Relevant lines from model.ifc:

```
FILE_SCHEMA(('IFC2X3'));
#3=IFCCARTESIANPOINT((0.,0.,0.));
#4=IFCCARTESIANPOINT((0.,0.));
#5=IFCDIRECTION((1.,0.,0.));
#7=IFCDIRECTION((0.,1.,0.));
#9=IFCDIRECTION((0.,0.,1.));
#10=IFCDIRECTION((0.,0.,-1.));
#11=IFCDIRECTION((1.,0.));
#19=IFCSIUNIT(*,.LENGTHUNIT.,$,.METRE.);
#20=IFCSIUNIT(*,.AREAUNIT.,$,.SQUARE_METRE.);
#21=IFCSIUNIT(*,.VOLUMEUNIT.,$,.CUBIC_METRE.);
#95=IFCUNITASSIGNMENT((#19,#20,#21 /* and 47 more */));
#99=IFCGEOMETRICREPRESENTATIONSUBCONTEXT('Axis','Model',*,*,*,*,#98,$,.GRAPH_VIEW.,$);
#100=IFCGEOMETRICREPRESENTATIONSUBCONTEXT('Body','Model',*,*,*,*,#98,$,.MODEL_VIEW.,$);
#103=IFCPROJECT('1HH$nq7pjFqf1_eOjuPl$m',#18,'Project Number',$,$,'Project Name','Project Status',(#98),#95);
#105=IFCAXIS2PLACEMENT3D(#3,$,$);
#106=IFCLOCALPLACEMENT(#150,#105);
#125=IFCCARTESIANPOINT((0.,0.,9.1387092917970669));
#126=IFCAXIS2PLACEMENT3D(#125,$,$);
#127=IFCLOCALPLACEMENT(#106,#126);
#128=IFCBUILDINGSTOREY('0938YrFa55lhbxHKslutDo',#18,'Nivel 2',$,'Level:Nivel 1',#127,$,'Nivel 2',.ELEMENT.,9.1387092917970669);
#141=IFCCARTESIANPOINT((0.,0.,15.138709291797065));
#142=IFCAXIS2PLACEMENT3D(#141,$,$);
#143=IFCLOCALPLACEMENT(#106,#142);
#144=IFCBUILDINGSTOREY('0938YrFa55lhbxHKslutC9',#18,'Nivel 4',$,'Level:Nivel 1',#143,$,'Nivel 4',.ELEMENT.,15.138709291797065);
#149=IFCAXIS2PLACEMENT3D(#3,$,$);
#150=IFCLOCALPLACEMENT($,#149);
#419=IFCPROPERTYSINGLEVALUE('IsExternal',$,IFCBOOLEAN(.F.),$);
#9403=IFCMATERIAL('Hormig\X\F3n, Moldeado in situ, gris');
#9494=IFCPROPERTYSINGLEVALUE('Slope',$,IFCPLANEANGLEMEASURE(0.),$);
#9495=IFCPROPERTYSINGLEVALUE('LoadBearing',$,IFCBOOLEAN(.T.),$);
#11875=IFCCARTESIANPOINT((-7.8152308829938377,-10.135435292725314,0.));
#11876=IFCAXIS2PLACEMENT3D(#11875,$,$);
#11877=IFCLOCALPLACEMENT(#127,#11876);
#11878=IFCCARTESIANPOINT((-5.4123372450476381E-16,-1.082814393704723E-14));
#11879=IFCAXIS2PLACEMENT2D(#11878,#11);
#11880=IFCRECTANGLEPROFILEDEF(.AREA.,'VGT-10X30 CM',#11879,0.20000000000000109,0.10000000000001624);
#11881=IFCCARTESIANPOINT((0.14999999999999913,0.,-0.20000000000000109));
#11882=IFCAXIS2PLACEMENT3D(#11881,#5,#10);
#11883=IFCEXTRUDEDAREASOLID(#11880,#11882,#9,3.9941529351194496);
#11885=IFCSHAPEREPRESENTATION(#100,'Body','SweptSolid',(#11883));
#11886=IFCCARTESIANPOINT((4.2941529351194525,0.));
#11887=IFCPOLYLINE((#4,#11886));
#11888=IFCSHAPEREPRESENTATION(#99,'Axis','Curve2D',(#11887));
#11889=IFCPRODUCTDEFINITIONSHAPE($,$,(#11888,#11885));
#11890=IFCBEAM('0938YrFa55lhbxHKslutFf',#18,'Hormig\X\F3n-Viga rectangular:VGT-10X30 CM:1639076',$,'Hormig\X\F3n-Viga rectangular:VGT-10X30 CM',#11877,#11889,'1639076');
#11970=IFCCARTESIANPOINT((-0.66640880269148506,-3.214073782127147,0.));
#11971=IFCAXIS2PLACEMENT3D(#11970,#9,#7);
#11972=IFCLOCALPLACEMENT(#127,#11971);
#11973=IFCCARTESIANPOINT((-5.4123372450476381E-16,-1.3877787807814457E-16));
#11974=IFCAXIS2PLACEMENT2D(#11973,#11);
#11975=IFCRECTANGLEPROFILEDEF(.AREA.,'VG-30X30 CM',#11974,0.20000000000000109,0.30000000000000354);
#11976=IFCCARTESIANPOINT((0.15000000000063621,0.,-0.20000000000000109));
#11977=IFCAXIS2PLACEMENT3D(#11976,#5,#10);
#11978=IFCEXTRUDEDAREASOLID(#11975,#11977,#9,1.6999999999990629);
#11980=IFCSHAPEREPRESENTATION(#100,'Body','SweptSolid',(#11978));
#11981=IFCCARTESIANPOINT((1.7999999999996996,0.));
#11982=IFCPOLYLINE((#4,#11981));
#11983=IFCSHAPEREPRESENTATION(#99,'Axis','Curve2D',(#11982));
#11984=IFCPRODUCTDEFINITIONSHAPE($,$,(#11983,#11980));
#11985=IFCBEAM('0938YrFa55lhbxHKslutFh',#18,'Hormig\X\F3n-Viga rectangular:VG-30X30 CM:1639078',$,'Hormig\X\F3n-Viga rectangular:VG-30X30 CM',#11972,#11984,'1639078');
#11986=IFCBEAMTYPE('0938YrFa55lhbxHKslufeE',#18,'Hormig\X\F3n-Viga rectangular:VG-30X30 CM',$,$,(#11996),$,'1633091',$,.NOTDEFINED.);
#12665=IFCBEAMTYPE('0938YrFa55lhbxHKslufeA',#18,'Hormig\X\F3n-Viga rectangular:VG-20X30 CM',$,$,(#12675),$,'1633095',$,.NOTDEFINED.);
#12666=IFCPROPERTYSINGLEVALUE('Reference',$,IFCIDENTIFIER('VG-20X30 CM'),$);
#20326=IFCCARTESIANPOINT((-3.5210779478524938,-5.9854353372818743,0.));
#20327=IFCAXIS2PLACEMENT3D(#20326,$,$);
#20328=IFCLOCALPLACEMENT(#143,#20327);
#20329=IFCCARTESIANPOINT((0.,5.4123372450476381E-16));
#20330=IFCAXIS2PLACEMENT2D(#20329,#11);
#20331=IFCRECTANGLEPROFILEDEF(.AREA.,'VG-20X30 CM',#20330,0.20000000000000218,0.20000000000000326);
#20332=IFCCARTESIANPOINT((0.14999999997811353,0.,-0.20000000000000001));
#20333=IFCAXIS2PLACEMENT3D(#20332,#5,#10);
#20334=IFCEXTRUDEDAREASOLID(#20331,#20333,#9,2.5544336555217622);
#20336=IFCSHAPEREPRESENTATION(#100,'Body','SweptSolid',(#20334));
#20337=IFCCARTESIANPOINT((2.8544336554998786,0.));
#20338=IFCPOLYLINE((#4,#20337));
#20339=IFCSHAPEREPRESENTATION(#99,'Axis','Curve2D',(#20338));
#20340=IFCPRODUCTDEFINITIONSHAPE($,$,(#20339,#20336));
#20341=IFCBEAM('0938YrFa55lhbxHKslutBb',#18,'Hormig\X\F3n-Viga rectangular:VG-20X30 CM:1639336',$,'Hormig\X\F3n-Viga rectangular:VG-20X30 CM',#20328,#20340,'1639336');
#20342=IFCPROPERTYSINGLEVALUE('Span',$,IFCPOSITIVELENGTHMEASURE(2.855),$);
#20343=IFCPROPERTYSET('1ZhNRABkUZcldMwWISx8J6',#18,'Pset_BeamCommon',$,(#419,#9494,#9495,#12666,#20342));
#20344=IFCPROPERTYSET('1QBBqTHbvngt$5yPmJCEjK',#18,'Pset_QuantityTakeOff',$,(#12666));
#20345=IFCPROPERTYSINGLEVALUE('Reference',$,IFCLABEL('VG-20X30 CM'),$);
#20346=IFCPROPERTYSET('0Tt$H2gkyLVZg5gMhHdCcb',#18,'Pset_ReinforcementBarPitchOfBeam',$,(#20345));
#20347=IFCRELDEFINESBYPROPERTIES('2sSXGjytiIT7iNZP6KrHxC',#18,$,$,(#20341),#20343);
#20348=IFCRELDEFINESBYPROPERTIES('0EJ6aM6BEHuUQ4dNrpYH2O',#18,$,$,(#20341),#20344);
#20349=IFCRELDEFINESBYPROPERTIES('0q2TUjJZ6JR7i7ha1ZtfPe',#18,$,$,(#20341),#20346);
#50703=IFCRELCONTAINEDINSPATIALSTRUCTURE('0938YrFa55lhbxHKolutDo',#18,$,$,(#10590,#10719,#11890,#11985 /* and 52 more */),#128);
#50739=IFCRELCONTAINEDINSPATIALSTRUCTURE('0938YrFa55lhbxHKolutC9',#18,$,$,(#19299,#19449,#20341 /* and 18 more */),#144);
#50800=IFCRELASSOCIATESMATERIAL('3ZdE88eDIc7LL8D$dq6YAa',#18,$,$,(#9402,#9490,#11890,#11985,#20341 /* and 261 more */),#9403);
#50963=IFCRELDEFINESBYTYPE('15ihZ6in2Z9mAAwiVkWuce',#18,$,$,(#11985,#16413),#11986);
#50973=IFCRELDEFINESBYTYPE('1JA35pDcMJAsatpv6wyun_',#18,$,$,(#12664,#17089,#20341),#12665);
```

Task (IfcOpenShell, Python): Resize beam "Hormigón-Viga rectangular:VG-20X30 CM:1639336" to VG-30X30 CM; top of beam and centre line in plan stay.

```python
import ifcopenshell
import ifcopenshell.api.pset
import ifcopenshell.api.type
import ifcopenshell.util.element
import ifcopenshell.util.representation

model = ifcopenshell.open("model.ifc")

member = model.by_guid("0938YrFa55lhbxHKslutBb")
source = next(p for p in model.by_type("IfcRectangleProfileDef") if p.ProfileName == "VG-30X30 CM")

body = ifcopenshell.util.representation.get_representation(member, "Model", "Body")
solid = body.Items[0]
old_profile = solid.SweptArea

# Copy the section's sizes but keep this member's own profile position.
profile = ifcopenshell.util.element.copy(model, source)
# Profiles are centred, so shift by half the change in depth to hold the top.
shift = (old_profile.XDim - profile.XDim) / 2
x, y = old_profile.Position.Location.Coordinates
up = (-1.0, 0.0)  # upwards, in the solid's own plane
location = model.createIfcCartesianPoint((x + up[0] * shift, y + up[1] * shift))
profile.Position = model.createIfcAxis2Placement2D(location, old_profile.Position.RefDirection)
solid.SweptArea = profile
if not model.get_total_inverses(old_profile):
    ifcopenshell.util.element.remove_deep2(model, old_profile)

new_type = model.by_id(11986)
ifcopenshell.api.type.assign_type(
    model, related_objects=[member], relating_type=new_type, should_map_representations=False
)
member.Name = member.Name.replace("VG-20X30 CM", "VG-30X30 CM")
member.ObjectType = "Hormigón-Viga rectangular:VG-30X30 CM"
pset = model.by_id(ifcopenshell.util.element.get_pset(member, "Pset_BeamCommon", should_inherit=False)["id"])
ifcopenshell.api.pset.edit_pset(model, pset=pset, properties={"Reference": "VG-30X30 CM"})
pset = model.by_id(ifcopenshell.util.element.get_pset(member, "Pset_QuantityTakeOff", should_inherit=False)["id"])
ifcopenshell.api.pset.edit_pset(model, pset=pset, properties={"Reference": "VG-30X30 CM"})
pset = model.by_id(ifcopenshell.util.element.get_pset(member, "Pset_ReinforcementBarPitchOfBeam", should_inherit=False)["id"])
ifcopenshell.api.pset.edit_pset(model, pset=pset, properties={"Reference": "VG-30X30 CM"})

print(solid.SweptArea)

model.write("model_updated.ifc")
```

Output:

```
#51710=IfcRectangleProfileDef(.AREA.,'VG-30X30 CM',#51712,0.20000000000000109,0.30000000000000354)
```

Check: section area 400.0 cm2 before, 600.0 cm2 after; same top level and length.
